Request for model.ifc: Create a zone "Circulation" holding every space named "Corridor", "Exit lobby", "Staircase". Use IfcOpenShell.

First a look at what the model holds.

```python
import ifcopenshell

model = ifcopenshell.open("model.ifc")
print(model.schema)
seen = {}
for space in model.by_type("IfcSpace"):
    seen[space.LongName] = seen.get(space.LongName, 0) + 1
for name, count in sorted(seen.items(), key=str):
    print(count, "x", name)
print("zones:", [z.Name for z in model.by_type("IfcZone")][:20])
```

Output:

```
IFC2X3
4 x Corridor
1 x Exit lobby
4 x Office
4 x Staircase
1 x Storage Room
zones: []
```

```python
import ifcopenshell
import ifcopenshell.api.group
import ifcopenshell.api.root

model = ifcopenshell.open("model.ifc")

names = {"Corridor", "Exit lobby", "Staircase"}
spaces = [s for s in model.by_type("IfcSpace") if s.LongName in names]

zone = ifcopenshell.api.root.create_entity(model, ifc_class="IfcZone", name="Circulation")
ifcopenshell.api.group.assign_group(model, products=spaces, group=zone)
print(len(spaces), "spaces in", zone.Name)

model.write("model_updated.ifc")
```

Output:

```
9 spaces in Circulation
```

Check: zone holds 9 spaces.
